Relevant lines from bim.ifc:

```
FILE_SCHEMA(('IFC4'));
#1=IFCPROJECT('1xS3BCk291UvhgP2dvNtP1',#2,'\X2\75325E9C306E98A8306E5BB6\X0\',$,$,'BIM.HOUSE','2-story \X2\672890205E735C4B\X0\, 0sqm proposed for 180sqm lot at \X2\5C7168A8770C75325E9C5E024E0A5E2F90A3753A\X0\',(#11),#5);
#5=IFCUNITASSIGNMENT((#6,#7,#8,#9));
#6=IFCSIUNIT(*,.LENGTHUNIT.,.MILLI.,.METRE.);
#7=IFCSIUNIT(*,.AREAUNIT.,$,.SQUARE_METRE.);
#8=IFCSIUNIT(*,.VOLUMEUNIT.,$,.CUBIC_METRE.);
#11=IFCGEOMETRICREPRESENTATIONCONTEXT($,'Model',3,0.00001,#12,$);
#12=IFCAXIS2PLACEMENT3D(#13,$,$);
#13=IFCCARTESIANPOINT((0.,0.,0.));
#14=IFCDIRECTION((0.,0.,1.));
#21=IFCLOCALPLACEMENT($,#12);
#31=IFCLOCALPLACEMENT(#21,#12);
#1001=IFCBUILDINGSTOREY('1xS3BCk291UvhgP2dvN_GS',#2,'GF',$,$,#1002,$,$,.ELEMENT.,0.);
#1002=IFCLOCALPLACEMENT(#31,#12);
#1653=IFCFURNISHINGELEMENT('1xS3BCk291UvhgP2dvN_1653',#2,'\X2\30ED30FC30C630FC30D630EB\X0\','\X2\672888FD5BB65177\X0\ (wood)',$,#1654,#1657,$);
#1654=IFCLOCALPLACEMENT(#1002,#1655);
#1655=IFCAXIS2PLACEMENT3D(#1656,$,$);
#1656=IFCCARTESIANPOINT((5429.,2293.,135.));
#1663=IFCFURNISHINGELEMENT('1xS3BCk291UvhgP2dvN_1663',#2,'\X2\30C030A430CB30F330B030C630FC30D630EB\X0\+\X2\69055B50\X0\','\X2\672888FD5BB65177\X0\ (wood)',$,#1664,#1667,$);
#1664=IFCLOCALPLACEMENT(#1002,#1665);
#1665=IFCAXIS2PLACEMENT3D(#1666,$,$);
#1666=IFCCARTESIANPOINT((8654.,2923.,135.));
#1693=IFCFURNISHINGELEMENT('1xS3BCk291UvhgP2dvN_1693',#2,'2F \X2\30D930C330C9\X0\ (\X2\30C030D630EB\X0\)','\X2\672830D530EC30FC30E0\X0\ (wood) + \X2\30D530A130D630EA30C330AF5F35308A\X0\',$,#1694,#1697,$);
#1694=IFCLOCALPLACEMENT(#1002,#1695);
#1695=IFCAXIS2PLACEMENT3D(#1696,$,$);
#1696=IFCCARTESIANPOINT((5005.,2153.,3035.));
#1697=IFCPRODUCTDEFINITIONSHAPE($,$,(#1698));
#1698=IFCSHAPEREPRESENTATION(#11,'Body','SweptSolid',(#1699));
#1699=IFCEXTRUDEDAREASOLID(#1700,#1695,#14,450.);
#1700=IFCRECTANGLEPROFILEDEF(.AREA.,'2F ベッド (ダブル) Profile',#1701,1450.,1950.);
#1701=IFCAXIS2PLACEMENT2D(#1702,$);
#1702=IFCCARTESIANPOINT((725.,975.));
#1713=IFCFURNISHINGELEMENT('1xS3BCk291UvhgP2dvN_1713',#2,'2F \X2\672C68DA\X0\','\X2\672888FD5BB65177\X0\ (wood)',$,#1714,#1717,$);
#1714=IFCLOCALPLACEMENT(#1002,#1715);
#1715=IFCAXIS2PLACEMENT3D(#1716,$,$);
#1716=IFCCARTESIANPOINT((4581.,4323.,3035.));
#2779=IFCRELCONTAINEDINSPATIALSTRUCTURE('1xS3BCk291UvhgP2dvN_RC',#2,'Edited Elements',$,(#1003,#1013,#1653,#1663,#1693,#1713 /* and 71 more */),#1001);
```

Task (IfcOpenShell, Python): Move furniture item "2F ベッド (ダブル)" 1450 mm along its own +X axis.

```python
import ifcopenshell
import ifcopenshell.api.geometry
import ifcopenshell.util.placement
import ifcopenshell.util.unit

model = ifcopenshell.open("bim.ifc")
unit_scale = ifcopenshell.util.unit.calculate_unit_scale(model)

item = model.by_guid("1xS3BCk291UvhgP2dvN_1693")
matrix = ifcopenshell.util.placement.get_local_placement(item.ObjectPlacement)
matrix[:3, 3] += matrix[:3, 0] * 1.45 / unit_scale
ifcopenshell.api.geometry.edit_object_placement(model, product=item, matrix=matrix, is_si=False)

print(ifcopenshell.util.placement.get_local_placement(item.ObjectPlacement).round(3) + 0.0)

model.write("bim_v2.ifc")
```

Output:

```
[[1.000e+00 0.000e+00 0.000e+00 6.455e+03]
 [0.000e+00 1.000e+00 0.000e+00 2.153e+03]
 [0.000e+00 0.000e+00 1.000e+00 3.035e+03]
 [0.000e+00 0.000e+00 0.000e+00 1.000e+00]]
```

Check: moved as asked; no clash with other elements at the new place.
